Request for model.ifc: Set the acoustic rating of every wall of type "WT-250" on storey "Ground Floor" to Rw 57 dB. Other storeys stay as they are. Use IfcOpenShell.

First a look at what the model holds.

```python
import ifcopenshell
import ifcopenshell.util.element

model = ifcopenshell.open("model.ifc")
print(model.schema)
storey = next(s for s in model.by_type("IfcBuildingStorey") if s.Name == "Ground Floor")
walls = [e for e in ifcopenshell.util.element.get_decomposition(storey) if e.is_a("IfcWall")]
seen = {}
for e in walls:
    element_type = ifcopenshell.util.element.get_type(e)
    key = (element_type.Name if element_type != e and element_type else None, ifcopenshell.util.element.get_pset(e, "Pset_WallCommon", "AcousticRating"))
    seen[key] = seen.get(key, 0) + 1
for (name, value), count in sorted(seen.items(), key=str):
    print(count, "x", name, "|", value)
```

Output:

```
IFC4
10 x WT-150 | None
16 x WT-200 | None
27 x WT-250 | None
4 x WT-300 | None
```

```python
import ifcopenshell
import ifcopenshell.api.pset
import ifcopenshell.util.element

model = ifcopenshell.open("model.ifc")

storey = next(s for s in model.by_type("IfcBuildingStorey") if s.Name == "Ground Floor")
walls = [e for e in ifcopenshell.util.element.get_decomposition(storey) if e.is_a("IfcWall")]

count = 0
for e in walls:
    element_type = ifcopenshell.util.element.get_type(e)
    if element_type in (None, e) or element_type.Name != "WT-250":
        continue
    # add_pset returns the element's existing set when there is one.
    pset = ifcopenshell.api.pset.add_pset(model, product=e, name="Pset_WallCommon")
    ifcopenshell.api.pset.edit_pset(model, pset=pset, properties={"AcousticRating": "Rw 57 dB"})
    count += 1

print(count, "walls updated")

model.write("model-out.ifc")
```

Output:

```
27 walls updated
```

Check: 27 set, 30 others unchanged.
